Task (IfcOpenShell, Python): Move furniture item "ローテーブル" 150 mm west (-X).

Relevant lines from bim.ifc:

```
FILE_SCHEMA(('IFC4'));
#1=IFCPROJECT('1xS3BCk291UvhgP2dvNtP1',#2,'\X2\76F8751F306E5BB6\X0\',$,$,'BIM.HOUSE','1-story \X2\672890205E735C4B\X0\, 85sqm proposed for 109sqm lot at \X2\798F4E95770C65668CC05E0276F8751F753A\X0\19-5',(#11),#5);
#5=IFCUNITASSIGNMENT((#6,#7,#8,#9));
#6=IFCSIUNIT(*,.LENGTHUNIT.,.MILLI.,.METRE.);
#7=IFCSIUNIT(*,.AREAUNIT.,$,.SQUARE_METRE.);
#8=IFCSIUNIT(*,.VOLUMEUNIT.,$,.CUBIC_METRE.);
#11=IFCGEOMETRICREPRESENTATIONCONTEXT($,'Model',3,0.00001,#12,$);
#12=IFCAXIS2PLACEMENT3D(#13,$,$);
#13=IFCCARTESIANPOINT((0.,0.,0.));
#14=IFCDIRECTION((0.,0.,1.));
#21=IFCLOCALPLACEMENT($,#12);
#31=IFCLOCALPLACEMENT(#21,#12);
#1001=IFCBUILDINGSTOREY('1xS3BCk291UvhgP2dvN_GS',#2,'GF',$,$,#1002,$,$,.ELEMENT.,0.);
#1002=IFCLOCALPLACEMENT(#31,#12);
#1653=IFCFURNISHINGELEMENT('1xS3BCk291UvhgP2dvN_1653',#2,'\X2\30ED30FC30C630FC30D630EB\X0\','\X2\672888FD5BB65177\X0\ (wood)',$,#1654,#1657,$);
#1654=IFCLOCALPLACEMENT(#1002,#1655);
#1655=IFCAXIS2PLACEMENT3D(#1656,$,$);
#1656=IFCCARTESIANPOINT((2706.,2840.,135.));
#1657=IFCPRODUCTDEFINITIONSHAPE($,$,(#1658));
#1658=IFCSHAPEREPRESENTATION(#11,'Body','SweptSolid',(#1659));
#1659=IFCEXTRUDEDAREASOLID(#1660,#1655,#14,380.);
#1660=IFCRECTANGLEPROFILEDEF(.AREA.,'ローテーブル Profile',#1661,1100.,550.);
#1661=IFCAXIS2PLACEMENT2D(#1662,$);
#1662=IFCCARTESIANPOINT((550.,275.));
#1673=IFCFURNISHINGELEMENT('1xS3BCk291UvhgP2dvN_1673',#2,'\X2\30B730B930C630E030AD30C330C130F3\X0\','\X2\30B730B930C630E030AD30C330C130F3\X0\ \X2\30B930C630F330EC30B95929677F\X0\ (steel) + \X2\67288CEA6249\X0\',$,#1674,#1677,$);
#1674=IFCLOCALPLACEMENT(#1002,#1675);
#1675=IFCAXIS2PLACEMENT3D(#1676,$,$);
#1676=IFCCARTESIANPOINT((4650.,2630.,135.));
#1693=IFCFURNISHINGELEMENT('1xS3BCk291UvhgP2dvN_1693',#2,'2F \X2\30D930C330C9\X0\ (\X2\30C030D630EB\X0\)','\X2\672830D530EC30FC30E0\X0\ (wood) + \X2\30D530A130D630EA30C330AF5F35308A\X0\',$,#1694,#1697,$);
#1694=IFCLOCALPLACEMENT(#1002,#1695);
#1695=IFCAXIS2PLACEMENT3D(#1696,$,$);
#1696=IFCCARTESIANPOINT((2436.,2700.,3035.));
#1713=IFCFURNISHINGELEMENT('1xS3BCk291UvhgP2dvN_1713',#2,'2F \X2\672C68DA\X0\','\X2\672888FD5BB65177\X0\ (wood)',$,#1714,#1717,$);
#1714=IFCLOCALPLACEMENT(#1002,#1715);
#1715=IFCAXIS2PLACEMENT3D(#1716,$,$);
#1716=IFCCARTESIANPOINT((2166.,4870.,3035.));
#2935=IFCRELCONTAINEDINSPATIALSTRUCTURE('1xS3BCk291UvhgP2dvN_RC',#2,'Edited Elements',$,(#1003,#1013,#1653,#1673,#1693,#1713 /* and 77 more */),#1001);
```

```python
import ifcopenshell
import ifcopenshell.api.geometry
import ifcopenshell.util.placement

model = ifcopenshell.open("bim.ifc")

item = model.by_guid("1xS3BCk291UvhgP2dvN_1653")
matrix = ifcopenshell.util.placement.get_local_placement(item.ObjectPlacement)
matrix[0, 3] -= 150.0
ifcopenshell.api.geometry.edit_object_placement(model, product=item, matrix=matrix, is_si=False)

print(ifcopenshell.util.placement.get_local_placement(item.ObjectPlacement).round(3) + 0.0)

model.write("bim_updated.ifc")
```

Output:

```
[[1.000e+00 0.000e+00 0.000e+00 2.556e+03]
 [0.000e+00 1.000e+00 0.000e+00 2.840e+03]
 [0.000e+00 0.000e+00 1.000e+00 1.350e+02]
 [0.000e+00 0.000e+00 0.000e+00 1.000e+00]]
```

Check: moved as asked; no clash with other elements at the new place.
